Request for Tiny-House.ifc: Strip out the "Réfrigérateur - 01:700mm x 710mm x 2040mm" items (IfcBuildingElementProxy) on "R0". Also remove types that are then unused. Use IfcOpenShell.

First a look at what the model holds.

```python
import ifcopenshell
import ifcopenshell.util.element

model = ifcopenshell.open("Tiny-House.ifc")
print(model.schema)
storey = next(s for s in model.by_type("IfcBuildingStorey") if s.Name == "R0")
proxies = [e for e in ifcopenshell.util.element.get_decomposition(storey) if e.is_a("IfcBuildingElementProxy")]
seen = {}
for e in proxies:
    element_type = ifcopenshell.util.element.get_type(e)
    name = element_type.Name if element_type not in (None, e) else None
    seen[name] = seen.get(name, 0) + 1
for name, count in sorted(seen.items(), key=str):
    print(count, "x", name)
```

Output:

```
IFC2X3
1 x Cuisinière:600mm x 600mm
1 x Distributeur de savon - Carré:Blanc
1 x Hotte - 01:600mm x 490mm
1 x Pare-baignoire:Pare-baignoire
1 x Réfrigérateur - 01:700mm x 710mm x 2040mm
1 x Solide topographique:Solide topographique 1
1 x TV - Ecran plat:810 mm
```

```python
import ifcopenshell
import ifcopenshell.api.root
import ifcopenshell.util.element

model = ifcopenshell.open("Tiny-House.ifc")

storey = next(s for s in model.by_type("IfcBuildingStorey") if s.Name == "R0")
proxies = [e for e in ifcopenshell.util.element.get_decomposition(storey) if e.is_a("IfcBuildingElementProxy")]
targets = [e for e in proxies if (t := ifcopenshell.util.element.get_type(e)) not in (None, e) and t.Name == "Réfrigérateur - 01:700mm x 710mm x 2040mm"]
types = {ifcopenshell.util.element.get_type(e) for e in targets} - {None, *targets}

for e in targets:
    ifcopenshell.api.root.remove_product(model, product=e)
print(len(targets), "removed")

unused = [t for t in types if not ifcopenshell.util.element.get_types(t)]
for t in unused:
    ifcopenshell.api.root.remove_product(model, product=t)
print(len(unused), "unused types removed")

model.write("Tiny-House-out.ifc")
```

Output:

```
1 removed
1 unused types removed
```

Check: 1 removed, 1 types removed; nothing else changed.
